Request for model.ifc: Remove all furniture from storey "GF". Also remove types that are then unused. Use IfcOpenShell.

First a look at what the model holds.

```python
import ifcopenshell
import ifcopenshell.util.element

model = ifcopenshell.open("model.ifc")
print(model.schema)
storey = next(s for s in model.by_type("IfcBuildingStorey") if s.Name == "GF")
furniture = [e for e in ifcopenshell.util.element.get_decomposition(storey) if e.is_a("IfcFurnishingElement")]
seen = {}
for e in furniture:
    element_type = ifcopenshell.util.element.get_type(e)
    name = element_type.Name if element_type not in (None, e) else None
    seen[name] = seen.get(name, 0) + 1
for name, count in sorted(seen.items(), key=str):
    print(count, "x", name)
```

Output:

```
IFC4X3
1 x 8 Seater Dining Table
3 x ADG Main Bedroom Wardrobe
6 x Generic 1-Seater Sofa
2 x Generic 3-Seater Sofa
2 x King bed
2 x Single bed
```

```python
import ifcopenshell
import ifcopenshell.api.root
import ifcopenshell.util.element

model = ifcopenshell.open("model.ifc")

storey = next(s for s in model.by_type("IfcBuildingStorey") if s.Name == "GF")
furniture = [e for e in ifcopenshell.util.element.get_decomposition(storey) if e.is_a("IfcFurnishingElement")]
types = {ifcopenshell.util.element.get_type(e) for e in furniture} - {None, *furniture}

for e in furniture:
    ifcopenshell.api.root.remove_product(model, product=e)
print(len(furniture), "removed")

unused = [t for t in types if not ifcopenshell.util.element.get_types(t)]
for t in unused:
    ifcopenshell.api.root.remove_product(model, product=t)
print(len(unused), "unused types removed")

model.write("model-out.ifc")
```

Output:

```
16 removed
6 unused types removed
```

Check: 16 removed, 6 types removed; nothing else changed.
